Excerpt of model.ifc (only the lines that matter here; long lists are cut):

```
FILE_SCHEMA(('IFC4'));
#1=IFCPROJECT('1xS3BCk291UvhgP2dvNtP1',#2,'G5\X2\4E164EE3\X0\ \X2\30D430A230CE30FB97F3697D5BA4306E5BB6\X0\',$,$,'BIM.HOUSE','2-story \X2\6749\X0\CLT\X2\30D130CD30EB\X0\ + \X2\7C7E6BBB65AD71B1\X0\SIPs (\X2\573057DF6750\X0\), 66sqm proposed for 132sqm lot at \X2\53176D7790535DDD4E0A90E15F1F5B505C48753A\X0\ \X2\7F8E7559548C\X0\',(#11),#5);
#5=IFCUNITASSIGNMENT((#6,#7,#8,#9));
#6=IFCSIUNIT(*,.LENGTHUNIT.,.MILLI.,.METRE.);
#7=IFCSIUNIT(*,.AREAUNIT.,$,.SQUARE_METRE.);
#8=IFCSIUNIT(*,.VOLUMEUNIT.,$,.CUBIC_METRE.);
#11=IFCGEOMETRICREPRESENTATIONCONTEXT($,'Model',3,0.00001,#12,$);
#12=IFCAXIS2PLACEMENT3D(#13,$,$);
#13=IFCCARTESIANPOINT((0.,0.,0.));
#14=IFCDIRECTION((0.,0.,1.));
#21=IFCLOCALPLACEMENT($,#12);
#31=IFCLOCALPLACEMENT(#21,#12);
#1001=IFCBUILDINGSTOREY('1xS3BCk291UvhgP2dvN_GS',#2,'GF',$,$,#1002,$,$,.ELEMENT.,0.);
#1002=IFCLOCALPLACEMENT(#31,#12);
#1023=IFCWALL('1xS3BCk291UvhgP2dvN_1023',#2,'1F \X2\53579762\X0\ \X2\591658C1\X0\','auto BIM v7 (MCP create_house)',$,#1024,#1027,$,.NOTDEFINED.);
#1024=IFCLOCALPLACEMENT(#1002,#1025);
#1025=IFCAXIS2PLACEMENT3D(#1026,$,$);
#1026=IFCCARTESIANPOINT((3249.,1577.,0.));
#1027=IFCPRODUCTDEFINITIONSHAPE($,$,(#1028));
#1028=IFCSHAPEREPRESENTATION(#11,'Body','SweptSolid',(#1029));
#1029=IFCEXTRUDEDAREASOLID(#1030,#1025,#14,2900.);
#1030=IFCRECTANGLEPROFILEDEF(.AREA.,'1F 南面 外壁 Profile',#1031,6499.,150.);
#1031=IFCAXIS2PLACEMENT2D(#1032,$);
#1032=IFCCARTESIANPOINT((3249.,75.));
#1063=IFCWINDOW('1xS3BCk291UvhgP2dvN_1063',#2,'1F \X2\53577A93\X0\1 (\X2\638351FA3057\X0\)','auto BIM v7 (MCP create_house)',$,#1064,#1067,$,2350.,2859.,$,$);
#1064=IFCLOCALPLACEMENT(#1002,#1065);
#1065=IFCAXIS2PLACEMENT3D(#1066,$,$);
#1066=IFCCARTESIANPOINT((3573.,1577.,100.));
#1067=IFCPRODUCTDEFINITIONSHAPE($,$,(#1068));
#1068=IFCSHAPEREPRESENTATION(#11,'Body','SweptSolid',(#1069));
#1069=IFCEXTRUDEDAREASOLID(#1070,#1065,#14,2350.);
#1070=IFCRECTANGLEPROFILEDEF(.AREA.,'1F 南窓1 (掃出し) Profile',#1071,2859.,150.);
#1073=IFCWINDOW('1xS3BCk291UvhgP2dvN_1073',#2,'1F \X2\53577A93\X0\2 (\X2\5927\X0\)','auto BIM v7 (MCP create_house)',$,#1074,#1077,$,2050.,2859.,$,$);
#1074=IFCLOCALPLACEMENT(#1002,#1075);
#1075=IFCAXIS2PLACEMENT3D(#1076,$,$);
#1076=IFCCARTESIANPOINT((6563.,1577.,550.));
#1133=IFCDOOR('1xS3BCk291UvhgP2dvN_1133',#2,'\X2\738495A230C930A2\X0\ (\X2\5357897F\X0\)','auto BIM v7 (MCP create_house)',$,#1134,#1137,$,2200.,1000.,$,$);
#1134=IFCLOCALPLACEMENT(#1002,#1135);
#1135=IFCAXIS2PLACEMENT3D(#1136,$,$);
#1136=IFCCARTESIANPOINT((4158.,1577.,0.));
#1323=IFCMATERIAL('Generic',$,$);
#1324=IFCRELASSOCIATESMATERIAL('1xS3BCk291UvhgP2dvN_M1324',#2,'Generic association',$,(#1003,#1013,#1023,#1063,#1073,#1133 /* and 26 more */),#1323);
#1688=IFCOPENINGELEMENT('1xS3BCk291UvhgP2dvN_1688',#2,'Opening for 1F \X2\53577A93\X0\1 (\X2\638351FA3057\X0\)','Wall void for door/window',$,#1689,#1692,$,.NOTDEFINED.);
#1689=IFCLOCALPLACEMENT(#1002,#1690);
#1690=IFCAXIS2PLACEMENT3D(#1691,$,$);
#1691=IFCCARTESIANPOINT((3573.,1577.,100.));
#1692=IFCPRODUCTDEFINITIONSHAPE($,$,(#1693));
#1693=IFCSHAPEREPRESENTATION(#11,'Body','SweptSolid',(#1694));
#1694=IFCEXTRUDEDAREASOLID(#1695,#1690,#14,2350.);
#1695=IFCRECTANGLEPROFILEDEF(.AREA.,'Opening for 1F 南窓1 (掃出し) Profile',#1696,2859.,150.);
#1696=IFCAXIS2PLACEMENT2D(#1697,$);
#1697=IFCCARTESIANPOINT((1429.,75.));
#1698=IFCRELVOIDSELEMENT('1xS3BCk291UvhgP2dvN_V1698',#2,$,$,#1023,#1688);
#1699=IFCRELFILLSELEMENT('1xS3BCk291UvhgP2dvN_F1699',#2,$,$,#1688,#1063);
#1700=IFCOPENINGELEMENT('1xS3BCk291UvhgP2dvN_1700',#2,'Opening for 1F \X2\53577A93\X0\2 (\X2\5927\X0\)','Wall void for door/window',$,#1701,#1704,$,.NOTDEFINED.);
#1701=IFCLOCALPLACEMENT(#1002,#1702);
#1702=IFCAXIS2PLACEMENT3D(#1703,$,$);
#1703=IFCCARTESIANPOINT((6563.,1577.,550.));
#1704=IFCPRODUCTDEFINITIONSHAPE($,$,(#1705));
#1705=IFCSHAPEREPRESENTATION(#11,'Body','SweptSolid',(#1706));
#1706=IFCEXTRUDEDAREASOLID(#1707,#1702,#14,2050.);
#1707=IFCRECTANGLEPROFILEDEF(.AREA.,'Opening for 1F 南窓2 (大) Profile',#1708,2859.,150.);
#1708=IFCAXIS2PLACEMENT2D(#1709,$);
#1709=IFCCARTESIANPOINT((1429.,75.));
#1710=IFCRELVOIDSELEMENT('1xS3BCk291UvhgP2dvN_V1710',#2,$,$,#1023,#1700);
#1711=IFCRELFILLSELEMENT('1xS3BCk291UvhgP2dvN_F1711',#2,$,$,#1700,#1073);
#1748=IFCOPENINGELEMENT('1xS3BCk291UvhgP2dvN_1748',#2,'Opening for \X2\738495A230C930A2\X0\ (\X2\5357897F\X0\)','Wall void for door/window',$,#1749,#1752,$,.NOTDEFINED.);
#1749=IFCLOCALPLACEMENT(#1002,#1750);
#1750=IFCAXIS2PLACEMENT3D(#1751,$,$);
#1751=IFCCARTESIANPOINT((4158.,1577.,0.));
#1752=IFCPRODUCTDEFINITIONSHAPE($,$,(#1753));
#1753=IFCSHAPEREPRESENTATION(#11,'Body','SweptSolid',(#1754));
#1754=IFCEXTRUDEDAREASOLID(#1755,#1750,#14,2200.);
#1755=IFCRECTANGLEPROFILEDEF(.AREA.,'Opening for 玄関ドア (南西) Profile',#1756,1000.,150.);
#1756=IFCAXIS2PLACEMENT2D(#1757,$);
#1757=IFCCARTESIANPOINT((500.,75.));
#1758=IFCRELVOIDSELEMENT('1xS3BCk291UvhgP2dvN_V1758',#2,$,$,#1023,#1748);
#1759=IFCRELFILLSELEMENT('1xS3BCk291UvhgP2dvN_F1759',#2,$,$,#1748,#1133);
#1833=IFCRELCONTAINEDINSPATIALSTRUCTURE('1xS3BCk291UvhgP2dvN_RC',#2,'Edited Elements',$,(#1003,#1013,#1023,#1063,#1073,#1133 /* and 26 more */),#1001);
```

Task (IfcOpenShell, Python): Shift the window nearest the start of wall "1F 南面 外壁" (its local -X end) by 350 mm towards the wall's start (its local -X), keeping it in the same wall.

```python
import ifcopenshell
import ifcopenshell.api.geometry
import ifcopenshell.util.placement
import ifcopenshell.util.unit

model = ifcopenshell.open("model.ifc")
unit_scale = ifcopenshell.util.unit.calculate_unit_scale(model)

window = model.by_guid("1xS3BCk291UvhgP2dvN_1063")
opening = window.FillsVoids[0].RelatingOpeningElement
wall = opening.VoidsElements[0].RelatingBuildingElement

wall_matrix = ifcopenshell.util.placement.get_local_placement(wall.ObjectPlacement)
shift = wall_matrix[:3, 0] * -0.35 / unit_scale
before = ifcopenshell.util.placement.get_local_placement(window.ObjectPlacement)[:3, 3].copy()

# The window is not placed relative to its opening, so move both.
for product in (opening, window):
    matrix = ifcopenshell.util.placement.get_local_placement(product.ObjectPlacement)
    matrix[:3, 3] += shift
    ifcopenshell.api.geometry.edit_object_placement(model, product=product, matrix=matrix, is_si=False)

after = ifcopenshell.util.placement.get_local_placement(window.ObjectPlacement)[:3, 3]
print("window moved by", (after - before).round(3) + 0.0)

model.write("model-out.ifc")
```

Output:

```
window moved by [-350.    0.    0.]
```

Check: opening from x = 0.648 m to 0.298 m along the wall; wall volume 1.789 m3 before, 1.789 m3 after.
